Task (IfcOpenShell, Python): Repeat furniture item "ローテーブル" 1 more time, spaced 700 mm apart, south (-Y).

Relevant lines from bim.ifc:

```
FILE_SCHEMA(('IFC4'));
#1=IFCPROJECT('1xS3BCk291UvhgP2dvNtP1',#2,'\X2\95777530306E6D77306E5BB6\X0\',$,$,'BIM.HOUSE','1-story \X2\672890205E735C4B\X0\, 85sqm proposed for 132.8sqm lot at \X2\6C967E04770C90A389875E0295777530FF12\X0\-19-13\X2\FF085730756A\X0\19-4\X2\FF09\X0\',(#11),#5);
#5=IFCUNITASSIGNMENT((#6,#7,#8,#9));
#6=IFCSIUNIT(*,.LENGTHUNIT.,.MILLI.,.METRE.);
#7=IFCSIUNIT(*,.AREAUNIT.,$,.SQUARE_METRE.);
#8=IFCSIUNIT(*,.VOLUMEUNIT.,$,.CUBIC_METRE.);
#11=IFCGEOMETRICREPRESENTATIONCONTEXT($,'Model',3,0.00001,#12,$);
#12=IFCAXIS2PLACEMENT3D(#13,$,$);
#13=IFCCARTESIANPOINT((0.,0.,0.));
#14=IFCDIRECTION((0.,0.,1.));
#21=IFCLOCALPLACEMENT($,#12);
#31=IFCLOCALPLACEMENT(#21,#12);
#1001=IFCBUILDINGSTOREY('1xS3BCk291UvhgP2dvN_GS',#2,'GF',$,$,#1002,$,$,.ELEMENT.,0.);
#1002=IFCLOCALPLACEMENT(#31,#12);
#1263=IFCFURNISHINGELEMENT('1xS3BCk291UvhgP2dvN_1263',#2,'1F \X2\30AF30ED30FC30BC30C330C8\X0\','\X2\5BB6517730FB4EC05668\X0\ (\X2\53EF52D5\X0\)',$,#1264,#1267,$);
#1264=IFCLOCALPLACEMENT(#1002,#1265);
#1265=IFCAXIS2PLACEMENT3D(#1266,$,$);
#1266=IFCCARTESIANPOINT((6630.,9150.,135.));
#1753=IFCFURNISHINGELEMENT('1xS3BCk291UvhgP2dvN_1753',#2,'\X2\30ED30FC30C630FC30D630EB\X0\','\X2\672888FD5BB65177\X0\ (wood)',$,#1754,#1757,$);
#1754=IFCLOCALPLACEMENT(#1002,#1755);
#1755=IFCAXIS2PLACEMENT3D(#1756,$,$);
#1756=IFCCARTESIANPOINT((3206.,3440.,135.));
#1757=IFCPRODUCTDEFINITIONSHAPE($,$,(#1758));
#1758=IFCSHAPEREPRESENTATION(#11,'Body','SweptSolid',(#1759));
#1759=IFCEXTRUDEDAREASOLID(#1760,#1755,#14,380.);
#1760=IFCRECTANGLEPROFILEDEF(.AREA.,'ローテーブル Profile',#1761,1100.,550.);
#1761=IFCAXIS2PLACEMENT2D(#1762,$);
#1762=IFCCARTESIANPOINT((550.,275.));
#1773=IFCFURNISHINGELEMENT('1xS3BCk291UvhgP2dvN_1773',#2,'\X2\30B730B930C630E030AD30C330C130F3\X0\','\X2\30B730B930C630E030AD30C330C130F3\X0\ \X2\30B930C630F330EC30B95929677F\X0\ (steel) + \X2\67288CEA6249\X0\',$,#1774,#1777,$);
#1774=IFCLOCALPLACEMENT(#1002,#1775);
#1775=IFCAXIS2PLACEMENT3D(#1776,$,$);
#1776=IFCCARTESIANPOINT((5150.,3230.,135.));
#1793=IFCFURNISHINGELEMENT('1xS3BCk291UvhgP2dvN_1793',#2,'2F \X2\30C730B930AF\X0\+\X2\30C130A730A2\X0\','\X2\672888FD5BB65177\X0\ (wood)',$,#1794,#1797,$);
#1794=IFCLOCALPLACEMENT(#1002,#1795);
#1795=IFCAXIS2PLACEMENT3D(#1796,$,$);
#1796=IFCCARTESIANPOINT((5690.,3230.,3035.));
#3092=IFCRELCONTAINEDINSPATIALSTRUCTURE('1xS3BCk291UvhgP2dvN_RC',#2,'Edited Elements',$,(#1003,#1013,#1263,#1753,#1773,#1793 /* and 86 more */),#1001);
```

```python
import numpy as np
import ifcopenshell
import ifcopenshell.api.geometry
import ifcopenshell.api.root
import ifcopenshell.util.element
import ifcopenshell.util.placement
import ifcopenshell.util.unit

model = ifcopenshell.open("bim.ifc")
unit_scale = ifcopenshell.util.unit.calculate_unit_scale(model)


def reuse_history(source, copy):
    """copy_class also copies each property set's owner history, people and application; keep the originals."""
    for rel in copy.IsDefinedBy:
        if rel.is_a("IfcRelDefinesByProperties") and (history := rel.RelatingPropertyDefinition.OwnerHistory):
            rel.RelatingPropertyDefinition.OwnerHistory = source.OwnerHistory
            ifcopenshell.util.element.remove_deep2(model, history)


source = model.by_id(1753)
base = ifcopenshell.util.placement.get_local_placement(source.ObjectPlacement)
step = np.array([0.0, -1.0, 0.0]) * 0.7 / unit_scale

for i in range(1, 2):
    copy = ifcopenshell.api.root.copy_class(model, product=source)
    copy.Representation = ifcopenshell.util.element.copy_deep(
        model, source.Representation, exclude=["IfcGeometricRepresentationContext", "IfcRepresentationMap"]
    )
    reuse_history(source, copy)
    matrix = base.copy()
    matrix[:3, 3] += i * step
    print("added at", matrix[:3, 3].round(3) + 0.0)
    ifcopenshell.api.geometry.edit_object_placement(model, product=copy, matrix=matrix, is_si=False)

model.write("bim_updated.ifc")
```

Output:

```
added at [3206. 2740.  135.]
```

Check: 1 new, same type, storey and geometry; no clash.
